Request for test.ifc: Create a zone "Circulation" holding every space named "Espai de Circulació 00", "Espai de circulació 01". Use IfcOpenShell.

First a look at what the model holds.

```python
import ifcopenshell

model = ifcopenshell.open("test.ifc")
print(model.schema)
seen = {}
for space in model.by_type("IfcSpace"):
    seen[space.LongName] = seen.get(space.LongName, 0) + 1
for name, count in sorted(seen.items(), key=str):
    print(count, "x", name)
print("zones:", [z.Name for z in model.by_type("IfcZone")][:20])
```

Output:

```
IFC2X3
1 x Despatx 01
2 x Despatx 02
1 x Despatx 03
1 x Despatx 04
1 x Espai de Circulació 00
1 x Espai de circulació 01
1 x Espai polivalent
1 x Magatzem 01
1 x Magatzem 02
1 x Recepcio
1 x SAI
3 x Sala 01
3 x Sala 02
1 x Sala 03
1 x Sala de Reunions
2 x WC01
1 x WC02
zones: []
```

```python
import ifcopenshell
import ifcopenshell.api.group
import ifcopenshell.api.root

model = ifcopenshell.open("test.ifc")

names = {"Espai de Circulació 00", "Espai de circulació 01"}
spaces = [s for s in model.by_type("IfcSpace") if s.LongName in names]

zone = ifcopenshell.api.root.create_entity(model, ifc_class="IfcZone", name="Circulation")
ifcopenshell.api.group.assign_group(model, products=spaces, group=zone)
print(len(spaces), "spaces in", zone.Name)

model.write("test_rev.ifc")
```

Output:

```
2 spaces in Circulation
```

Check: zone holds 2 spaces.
